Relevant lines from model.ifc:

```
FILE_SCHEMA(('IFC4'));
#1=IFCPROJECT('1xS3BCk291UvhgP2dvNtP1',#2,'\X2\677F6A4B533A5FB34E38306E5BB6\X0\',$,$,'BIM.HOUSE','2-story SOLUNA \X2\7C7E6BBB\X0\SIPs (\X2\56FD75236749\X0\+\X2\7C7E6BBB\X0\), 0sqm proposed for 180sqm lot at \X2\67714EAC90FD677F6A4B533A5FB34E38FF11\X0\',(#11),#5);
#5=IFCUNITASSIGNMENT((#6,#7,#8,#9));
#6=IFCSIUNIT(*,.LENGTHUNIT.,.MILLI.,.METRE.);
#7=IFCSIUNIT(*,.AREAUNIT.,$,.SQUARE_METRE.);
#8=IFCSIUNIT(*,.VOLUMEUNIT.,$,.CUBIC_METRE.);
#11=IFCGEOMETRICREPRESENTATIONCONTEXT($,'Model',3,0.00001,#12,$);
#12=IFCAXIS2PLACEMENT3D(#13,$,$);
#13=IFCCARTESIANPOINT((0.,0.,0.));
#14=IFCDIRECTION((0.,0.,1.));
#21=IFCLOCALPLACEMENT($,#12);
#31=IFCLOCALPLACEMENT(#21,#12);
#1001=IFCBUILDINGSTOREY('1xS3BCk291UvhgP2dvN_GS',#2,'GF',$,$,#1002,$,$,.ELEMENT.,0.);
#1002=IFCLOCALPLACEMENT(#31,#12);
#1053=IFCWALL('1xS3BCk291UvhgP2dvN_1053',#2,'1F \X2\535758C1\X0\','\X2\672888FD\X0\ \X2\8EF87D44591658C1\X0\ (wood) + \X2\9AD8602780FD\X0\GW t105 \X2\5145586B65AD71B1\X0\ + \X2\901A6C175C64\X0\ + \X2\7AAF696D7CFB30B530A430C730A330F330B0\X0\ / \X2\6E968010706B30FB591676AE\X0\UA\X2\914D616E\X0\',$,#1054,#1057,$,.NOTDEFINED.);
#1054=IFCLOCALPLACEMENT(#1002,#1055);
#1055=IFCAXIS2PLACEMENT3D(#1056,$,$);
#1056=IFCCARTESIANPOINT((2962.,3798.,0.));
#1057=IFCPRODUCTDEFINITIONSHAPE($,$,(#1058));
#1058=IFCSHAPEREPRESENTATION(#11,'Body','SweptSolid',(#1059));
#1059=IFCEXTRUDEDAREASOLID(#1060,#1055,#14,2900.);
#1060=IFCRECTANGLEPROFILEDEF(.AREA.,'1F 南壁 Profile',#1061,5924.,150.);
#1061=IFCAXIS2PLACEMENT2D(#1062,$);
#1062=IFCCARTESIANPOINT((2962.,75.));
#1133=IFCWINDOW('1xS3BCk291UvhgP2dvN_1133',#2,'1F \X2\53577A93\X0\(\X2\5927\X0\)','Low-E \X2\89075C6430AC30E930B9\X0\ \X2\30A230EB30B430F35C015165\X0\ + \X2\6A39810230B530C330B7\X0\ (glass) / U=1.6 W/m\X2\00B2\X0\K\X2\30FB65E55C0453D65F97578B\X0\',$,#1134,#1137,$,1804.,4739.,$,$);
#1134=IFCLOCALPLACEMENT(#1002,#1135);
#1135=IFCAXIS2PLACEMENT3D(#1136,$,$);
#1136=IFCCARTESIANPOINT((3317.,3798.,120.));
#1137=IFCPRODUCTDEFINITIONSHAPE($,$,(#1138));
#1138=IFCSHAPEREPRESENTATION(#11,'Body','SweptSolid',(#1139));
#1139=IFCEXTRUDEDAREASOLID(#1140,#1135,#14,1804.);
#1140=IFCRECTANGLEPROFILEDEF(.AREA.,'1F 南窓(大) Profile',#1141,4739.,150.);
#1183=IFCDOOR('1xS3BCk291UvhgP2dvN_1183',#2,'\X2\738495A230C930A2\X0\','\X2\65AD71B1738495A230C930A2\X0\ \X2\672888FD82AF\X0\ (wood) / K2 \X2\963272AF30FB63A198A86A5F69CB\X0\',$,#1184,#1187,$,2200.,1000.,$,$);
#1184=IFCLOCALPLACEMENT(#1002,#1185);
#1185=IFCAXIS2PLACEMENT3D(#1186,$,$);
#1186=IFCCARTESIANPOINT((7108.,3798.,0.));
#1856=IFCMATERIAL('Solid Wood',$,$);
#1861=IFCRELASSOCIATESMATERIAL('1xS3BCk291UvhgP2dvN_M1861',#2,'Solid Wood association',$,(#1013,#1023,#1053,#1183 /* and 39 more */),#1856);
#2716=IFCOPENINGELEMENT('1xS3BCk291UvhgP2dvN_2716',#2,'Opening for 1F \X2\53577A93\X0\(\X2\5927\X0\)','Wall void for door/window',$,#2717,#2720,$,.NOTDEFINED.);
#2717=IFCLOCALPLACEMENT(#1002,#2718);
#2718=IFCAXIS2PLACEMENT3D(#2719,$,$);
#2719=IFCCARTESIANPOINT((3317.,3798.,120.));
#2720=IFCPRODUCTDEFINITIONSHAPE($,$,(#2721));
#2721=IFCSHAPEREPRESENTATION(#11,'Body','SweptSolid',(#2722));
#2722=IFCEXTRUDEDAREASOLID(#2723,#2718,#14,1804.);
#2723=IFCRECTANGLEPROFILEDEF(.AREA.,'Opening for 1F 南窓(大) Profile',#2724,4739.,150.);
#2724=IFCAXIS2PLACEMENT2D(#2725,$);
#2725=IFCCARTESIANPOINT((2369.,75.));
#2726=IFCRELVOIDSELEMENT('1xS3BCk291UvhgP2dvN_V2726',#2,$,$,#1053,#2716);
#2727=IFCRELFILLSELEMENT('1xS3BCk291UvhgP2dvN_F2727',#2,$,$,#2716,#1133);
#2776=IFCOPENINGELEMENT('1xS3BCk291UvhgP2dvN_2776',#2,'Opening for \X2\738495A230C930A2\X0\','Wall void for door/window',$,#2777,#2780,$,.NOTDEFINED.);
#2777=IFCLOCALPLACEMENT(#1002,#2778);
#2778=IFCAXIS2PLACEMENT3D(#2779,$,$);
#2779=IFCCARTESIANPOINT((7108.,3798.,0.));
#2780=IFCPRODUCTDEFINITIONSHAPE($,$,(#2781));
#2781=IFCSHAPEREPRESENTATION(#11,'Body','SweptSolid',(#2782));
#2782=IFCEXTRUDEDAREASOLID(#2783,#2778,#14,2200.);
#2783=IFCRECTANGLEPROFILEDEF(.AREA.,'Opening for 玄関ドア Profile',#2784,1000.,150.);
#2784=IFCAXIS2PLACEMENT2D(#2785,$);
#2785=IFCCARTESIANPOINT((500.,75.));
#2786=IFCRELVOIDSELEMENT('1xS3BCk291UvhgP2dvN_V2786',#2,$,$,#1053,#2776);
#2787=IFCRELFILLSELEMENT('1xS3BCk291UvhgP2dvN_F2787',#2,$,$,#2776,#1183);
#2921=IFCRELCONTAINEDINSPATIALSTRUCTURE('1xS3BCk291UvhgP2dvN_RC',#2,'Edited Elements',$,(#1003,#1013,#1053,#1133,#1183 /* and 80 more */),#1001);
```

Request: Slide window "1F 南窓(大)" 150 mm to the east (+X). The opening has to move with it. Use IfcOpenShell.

```python
import ifcopenshell
import ifcopenshell.api.geometry
import ifcopenshell.util.placement

model = ifcopenshell.open("model.ifc")

window = model.by_guid("1xS3BCk291UvhgP2dvN_1133")
opening = window.FillsVoids[0].RelatingOpeningElement
wall = opening.VoidsElements[0].RelatingBuildingElement

wall_matrix = ifcopenshell.util.placement.get_local_placement(wall.ObjectPlacement)
shift = wall_matrix[:3, 0] * 150.0
before = ifcopenshell.util.placement.get_local_placement(window.ObjectPlacement)[:3, 3].copy()

# The window is not placed relative to its opening, so move both.
for product in (opening, window):
    matrix = ifcopenshell.util.placement.get_local_placement(product.ObjectPlacement)
    matrix[:3, 3] += shift
    ifcopenshell.api.geometry.edit_object_placement(model, product=product, matrix=matrix, is_si=False)

after = ifcopenshell.util.placement.get_local_placement(window.ObjectPlacement)[:3, 3]
print("window moved by", (after - before).round(3) + 0.0)

model.write("model_v2.ifc")
```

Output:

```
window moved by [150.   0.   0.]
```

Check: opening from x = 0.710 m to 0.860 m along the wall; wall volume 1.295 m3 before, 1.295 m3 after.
